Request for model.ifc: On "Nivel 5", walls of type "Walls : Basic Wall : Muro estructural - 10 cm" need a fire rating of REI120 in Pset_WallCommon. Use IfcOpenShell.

First a look at what the model holds.

```python
import ifcopenshell
import ifcopenshell.util.element

model = ifcopenshell.open("model.ifc")
print(model.schema)
storey = next(s for s in model.by_type("IfcBuildingStorey") if s.Name == "Nivel 5")
walls = [e for e in ifcopenshell.util.element.get_decomposition(storey) if e.is_a("IfcWall")]
seen = {}
for e in walls:
    element_type = ifcopenshell.util.element.get_type(e)
    key = (element_type.Name if element_type != e and element_type else None, ifcopenshell.util.element.get_pset(e, "Pset_WallCommon", "FireRating"))
    seen[key] = seen.get(key, 0) + 1
for (name, value), count in sorted(seen.items(), key=str):
    print(count, "x", name, "|", value)
```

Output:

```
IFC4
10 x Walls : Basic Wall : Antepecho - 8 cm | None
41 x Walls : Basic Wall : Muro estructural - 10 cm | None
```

```python
import ifcopenshell
import ifcopenshell.api.pset
import ifcopenshell.util.element

model = ifcopenshell.open("model.ifc")

storey = next(s for s in model.by_type("IfcBuildingStorey") if s.Name == "Nivel 5")
walls = [e for e in ifcopenshell.util.element.get_decomposition(storey) if e.is_a("IfcWall")]

count = 0
for e in walls:
    element_type = ifcopenshell.util.element.get_type(e)
    if element_type in (None, e) or element_type.Name != "Walls : Basic Wall : Muro estructural - 10 cm":
        continue
    # add_pset returns the element's existing set when there is one.
    pset = ifcopenshell.api.pset.add_pset(model, product=e, name="Pset_WallCommon")
    ifcopenshell.api.pset.edit_pset(model, pset=pset, properties={"FireRating": "REI120"})
    count += 1

print(count, "walls updated")

model.write("model_v2.ifc")
```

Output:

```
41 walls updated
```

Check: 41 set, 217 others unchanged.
